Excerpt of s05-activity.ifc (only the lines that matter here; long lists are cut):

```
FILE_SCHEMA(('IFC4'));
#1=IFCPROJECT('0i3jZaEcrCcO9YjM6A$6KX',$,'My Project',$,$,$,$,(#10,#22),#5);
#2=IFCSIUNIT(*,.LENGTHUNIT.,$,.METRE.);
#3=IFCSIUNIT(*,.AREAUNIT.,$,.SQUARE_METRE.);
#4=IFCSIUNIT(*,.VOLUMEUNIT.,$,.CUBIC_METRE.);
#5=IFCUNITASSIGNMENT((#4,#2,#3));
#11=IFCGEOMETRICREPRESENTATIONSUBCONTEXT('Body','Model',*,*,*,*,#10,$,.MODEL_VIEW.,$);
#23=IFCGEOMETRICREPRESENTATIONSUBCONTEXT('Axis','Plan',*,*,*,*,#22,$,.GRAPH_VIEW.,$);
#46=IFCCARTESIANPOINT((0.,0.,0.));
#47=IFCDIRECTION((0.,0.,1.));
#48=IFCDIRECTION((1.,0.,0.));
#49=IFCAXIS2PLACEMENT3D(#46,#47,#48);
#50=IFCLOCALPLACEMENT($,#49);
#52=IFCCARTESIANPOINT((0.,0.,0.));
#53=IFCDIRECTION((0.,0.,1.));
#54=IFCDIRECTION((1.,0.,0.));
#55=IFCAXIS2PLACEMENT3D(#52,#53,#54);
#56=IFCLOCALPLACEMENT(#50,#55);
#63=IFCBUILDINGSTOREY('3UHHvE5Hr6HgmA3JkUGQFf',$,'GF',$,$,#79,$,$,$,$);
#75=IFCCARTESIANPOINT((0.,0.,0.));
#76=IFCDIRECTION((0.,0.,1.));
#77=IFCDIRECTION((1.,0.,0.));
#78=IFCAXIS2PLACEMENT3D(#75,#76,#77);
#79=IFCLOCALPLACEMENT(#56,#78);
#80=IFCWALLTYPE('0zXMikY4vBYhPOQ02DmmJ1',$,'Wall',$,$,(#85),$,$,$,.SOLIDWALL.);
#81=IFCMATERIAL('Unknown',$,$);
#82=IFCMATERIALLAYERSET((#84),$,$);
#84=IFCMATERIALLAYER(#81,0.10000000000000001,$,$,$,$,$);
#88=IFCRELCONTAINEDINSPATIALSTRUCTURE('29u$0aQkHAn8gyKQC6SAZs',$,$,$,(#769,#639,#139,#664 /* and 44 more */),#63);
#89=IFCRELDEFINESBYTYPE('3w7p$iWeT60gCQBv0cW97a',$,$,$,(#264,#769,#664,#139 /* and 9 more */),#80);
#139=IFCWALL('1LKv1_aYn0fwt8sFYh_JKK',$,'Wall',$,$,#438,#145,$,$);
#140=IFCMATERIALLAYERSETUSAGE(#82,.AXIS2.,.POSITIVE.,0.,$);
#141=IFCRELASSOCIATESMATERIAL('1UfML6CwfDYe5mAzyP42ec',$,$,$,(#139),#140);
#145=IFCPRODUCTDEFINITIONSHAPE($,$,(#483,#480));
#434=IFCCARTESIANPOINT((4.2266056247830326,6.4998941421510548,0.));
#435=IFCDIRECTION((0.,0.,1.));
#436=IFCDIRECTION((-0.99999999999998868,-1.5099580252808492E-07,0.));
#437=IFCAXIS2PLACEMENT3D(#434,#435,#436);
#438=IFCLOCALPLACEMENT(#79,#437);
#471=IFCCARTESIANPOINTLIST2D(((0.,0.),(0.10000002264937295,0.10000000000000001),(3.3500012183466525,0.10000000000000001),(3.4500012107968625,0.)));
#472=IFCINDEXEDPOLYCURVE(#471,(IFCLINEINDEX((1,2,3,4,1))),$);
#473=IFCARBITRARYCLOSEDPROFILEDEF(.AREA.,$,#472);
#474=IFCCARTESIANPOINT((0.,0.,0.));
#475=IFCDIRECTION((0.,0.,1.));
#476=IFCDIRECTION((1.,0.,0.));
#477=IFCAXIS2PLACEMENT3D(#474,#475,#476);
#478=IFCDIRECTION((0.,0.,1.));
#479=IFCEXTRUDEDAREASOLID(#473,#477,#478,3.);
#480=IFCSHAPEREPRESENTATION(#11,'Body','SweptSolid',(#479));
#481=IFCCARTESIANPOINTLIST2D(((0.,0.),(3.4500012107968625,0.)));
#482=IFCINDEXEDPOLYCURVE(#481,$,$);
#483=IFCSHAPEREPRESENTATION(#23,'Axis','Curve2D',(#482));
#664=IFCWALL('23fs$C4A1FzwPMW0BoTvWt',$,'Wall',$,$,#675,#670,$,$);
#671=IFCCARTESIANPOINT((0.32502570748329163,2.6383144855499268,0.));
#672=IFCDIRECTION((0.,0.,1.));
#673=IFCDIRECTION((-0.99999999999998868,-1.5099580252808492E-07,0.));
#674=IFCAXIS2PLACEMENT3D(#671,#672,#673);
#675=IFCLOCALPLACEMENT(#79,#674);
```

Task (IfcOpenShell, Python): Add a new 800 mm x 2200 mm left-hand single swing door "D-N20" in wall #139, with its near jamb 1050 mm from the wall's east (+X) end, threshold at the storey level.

```python
import numpy as np
import ifcopenshell
import ifcopenshell.api.feature
import ifcopenshell.api.geometry
import ifcopenshell.api.root
import ifcopenshell.api.spatial
import ifcopenshell.geom
import ifcopenshell.util.element
import ifcopenshell.util.placement
import ifcopenshell.util.representation
import ifcopenshell.util.shape
import ifcopenshell.util.unit

model = ifcopenshell.open("s05-activity.ifc")
unit_scale = ifcopenshell.util.unit.calculate_unit_scale(model)
settings = ifcopenshell.geom.settings()


def volume(element):
    """Net volume in cubic metres, openings subtracted."""
    shape = ifcopenshell.geom.create_shape(settings, element)
    return ifcopenshell.util.shape.get_volume(shape.geometry)


wall = model.by_guid("1LKv1_aYn0fwt8sFYh_JKK")
storey = ifcopenshell.util.element.get_container(wall, ifc_class="IfcBuildingStorey")
context = ifcopenshell.util.representation.get_context(model, "Model", "Body", "MODEL_VIEW")
before = volume(wall)

width, height, from_end, sill = 0.8, 2.2, 1.05, 0.0  # metres

# The wall runs along its own X axis, and the end named is its -X end.
wall_shape = ifcopenshell.geom.create_shape(settings, wall)
x, y, z = ifcopenshell.util.shape.get_vertices(wall_shape.geometry).T
start = x.min() + from_end
face, thickness = float(y.min()), float(y.max() - y.min())
wall_matrix = ifcopenshell.util.placement.get_local_placement(wall.ObjectPlacement)
level = ifcopenshell.util.placement.get_local_placement(storey.ObjectPlacement)[2, 3]


def in_wall(x, y):
    """Placement at x, y metres in the wall's axes, at sill height."""
    matrix = wall_matrix.copy()
    matrix[:, 3] = wall_matrix @ np.array([x / unit_scale, y / unit_scale, 0.0, 1.0])
    matrix[2, 3] = level + sill / unit_scale
    return matrix


# Opening: a box that overshoots both wall faces by 50 mm.
opening = ifcopenshell.api.root.create_entity(model, ifc_class="IfcOpeningElement", predefined_type="OPENING")
box = ifcopenshell.api.geometry.add_wall_representation(
    model, context=context, length=width, height=height, thickness=thickness + 0.1
)
ifcopenshell.api.geometry.assign_representation(model, product=opening, representation=box)
ifcopenshell.api.geometry.edit_object_placement(model, product=opening, matrix=in_wall(start, face - 0.05), is_si=False)
ifcopenshell.api.feature.add_feature(model, feature=opening, element=wall)

door = ifcopenshell.api.root.create_entity(model, ifc_class="IfcDoor", name="D-N20", predefined_type="DOOR")
door.OverallWidth, door.OverallHeight = width / unit_scale, height / unit_scale
door.OperationType = "SINGLE_SWING_LEFT"
body = ifcopenshell.api.geometry.add_door_representation(
    model,
    context=context,
    overall_width=door.OverallWidth,
    overall_height=door.OverallHeight,
    operation_type="SINGLE_SWING_LEFT",
    lining_properties={"LiningDepth": thickness / unit_scale, "ThresholdDepth": thickness / unit_scale},
)
ifcopenshell.api.geometry.assign_representation(model, product=door, representation=body)
ifcopenshell.api.spatial.assign_container(model, products=[door], relating_structure=storey)
ifcopenshell.api.feature.add_filling(model, opening=opening, element=door)

# The lining spans the wall, so the door starts at the wall face.
ifcopenshell.api.geometry.edit_object_placement(model, product=door, matrix=in_wall(start, face), is_si=False)

after = volume(wall)

print(f"wall volume {before:.3f} -> {after:.3f} m3")

model.write("s05-activity-out.ifc")
```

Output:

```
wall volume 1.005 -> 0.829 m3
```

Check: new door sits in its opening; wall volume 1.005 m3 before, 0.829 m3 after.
